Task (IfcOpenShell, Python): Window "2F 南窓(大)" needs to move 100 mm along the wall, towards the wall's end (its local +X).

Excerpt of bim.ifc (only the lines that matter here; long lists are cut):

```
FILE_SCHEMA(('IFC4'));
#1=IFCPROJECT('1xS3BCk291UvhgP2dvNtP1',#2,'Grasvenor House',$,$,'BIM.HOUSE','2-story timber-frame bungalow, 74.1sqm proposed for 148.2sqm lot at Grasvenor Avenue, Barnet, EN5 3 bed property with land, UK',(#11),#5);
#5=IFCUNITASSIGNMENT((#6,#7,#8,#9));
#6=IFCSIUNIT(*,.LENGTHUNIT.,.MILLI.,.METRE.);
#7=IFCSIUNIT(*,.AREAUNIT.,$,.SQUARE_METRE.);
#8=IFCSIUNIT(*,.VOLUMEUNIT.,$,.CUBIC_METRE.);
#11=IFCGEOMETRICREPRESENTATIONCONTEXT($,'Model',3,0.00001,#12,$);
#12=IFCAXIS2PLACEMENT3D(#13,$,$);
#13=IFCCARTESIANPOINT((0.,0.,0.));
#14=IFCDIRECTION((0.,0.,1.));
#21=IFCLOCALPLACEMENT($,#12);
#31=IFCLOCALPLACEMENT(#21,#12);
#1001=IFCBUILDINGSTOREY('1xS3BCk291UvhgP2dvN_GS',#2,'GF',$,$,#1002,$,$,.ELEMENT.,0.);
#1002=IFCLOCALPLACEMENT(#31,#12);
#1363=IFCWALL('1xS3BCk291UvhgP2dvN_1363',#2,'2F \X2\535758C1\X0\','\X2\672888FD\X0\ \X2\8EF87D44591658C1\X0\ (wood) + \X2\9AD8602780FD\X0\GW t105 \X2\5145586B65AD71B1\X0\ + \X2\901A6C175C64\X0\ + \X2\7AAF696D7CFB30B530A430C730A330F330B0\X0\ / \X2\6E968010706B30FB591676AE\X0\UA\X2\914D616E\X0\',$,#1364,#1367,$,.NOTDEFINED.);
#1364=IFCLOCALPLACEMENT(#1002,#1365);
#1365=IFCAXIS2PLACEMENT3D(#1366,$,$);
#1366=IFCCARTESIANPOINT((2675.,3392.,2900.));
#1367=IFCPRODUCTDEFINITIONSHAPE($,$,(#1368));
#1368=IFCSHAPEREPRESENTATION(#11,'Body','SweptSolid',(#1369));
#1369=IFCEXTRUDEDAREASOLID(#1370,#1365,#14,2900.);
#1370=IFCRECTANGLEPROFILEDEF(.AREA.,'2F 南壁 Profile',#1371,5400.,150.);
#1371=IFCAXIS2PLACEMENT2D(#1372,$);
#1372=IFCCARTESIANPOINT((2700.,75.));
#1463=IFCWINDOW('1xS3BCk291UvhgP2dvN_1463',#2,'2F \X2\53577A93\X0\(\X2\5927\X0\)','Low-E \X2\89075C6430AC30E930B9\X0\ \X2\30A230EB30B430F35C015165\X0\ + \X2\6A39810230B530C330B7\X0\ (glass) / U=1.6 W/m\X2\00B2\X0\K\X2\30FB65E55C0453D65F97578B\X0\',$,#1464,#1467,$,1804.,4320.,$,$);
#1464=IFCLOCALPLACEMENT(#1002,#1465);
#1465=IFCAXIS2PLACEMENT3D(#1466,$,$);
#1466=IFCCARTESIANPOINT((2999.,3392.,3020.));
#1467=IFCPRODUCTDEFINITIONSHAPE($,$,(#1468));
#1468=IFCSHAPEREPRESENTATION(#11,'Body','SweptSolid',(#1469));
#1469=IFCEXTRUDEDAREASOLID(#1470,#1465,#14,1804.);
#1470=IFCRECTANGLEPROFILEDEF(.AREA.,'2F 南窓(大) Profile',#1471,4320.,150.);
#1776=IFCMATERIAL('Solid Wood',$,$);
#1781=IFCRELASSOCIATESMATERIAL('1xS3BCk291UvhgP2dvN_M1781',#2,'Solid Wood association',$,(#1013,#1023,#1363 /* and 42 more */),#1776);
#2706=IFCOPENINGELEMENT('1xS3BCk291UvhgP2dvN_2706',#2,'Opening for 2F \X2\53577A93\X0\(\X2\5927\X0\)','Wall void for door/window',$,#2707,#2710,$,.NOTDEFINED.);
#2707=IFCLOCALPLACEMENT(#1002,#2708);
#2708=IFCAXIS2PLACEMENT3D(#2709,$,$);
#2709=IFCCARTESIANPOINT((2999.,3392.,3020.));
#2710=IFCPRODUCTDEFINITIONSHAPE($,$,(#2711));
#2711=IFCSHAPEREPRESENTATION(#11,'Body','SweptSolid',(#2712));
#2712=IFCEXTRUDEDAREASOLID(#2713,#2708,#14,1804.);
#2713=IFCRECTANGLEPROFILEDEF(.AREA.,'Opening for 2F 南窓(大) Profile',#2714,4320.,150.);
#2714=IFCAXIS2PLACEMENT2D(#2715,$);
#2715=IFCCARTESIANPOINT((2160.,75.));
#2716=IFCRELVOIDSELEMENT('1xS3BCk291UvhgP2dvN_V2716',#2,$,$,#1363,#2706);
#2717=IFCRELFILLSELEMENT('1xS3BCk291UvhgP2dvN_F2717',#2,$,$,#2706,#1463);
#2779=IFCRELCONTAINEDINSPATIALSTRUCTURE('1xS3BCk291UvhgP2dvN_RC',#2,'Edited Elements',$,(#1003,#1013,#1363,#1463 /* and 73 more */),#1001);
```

```python
import ifcopenshell
import ifcopenshell.api.geometry
import ifcopenshell.util.placement

model = ifcopenshell.open("bim.ifc")

window = model.by_guid("1xS3BCk291UvhgP2dvN_1463")
opening = window.FillsVoids[0].RelatingOpeningElement
wall = opening.VoidsElements[0].RelatingBuildingElement

wall_matrix = ifcopenshell.util.placement.get_local_placement(wall.ObjectPlacement)
shift = wall_matrix[:3, 0] * 100.0
before = ifcopenshell.util.placement.get_local_placement(window.ObjectPlacement)[:3, 3].copy()

# The window is not placed relative to its opening, so move both.
for product in (opening, window):
    matrix = ifcopenshell.util.placement.get_local_placement(product.ObjectPlacement)
    matrix[:3, 3] += shift
    ifcopenshell.api.geometry.edit_object_placement(model, product=product, matrix=matrix, is_si=False)

after = ifcopenshell.util.placement.get_local_placement(window.ObjectPlacement)[:3, 3]
print("window moved by", (after - before).round(3) + 0.0)

model.write("bim_updated.ifc")
```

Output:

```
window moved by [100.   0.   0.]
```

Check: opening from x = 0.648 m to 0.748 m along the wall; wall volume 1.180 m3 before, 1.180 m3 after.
